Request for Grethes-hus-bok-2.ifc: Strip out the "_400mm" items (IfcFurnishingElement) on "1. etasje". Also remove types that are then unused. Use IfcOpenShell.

First a look at what the model holds.

```python
import ifcopenshell
import ifcopenshell.util.element

model = ifcopenshell.open("Grethes-hus-bok-2.ifc")
print(model.schema)
storey = next(s for s in model.by_type("IfcBuildingStorey") if s.Name == "1. etasje")
furniture = [e for e in ifcopenshell.util.element.get_decomposition(storey) if e.is_a("IfcFurnishingElement")]
seen = {}
for e in furniture:
    element_type = ifcopenshell.util.element.get_type(e)
    name = element_type.Name if element_type not in (None, e) else None
    seen[name] = seen.get(name, 0) + 1
for name, count in sorted(seen.items(), key=str):
    print(count, "x", name)
```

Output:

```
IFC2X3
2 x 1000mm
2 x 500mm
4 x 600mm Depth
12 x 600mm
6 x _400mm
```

```python
import ifcopenshell
import ifcopenshell.api.root
import ifcopenshell.util.element

model = ifcopenshell.open("Grethes-hus-bok-2.ifc")

storey = next(s for s in model.by_type("IfcBuildingStorey") if s.Name == "1. etasje")
furniture = [e for e in ifcopenshell.util.element.get_decomposition(storey) if e.is_a("IfcFurnishingElement")]
targets = [e for e in furniture if (t := ifcopenshell.util.element.get_type(e)) not in (None, e) and t.Name == "_400mm"]
types = {ifcopenshell.util.element.get_type(e) for e in targets} - {None, *targets}

for e in targets:
    ifcopenshell.api.root.remove_product(model, product=e)
print(len(targets), "removed")

unused = [t for t in types if not ifcopenshell.util.element.get_types(t)]
for t in unused:
    ifcopenshell.api.root.remove_product(model, product=t)
print(len(unused), "unused types removed")

model.write("Grethes-hus-bok-2-out.ifc")
```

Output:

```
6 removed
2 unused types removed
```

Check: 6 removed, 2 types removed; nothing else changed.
